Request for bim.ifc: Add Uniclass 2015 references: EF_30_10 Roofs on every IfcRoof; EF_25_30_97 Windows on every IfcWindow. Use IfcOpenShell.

First a look at what the model holds.

```python
import ifcopenshell

model = ifcopenshell.open("bim.ifc")
print(model.schema)
print("classifications:", [c.Name for c in model.by_type("IfcClassification")])
for ifc_class in ("IfcDoor", "IfcRoof", "IfcStair", "IfcWall", "IfcWindow"):
    print(ifc_class, len(model.by_type(ifc_class)))
```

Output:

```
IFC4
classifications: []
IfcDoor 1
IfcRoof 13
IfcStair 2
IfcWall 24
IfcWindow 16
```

```python
import ifcopenshell
import ifcopenshell.api.classification

model = ifcopenshell.open("bim.ifc")

system = ifcopenshell.api.classification.add_classification(model, classification="Uniclass 2015")

codes = {
    "IfcRoof": ("EF_30_10", "Roofs"),
    "IfcWindow": ("EF_25_30_97", "Windows"),
}
for ifc_class, (code, name) in codes.items():
    products = model.by_type(ifc_class)
    ifcopenshell.api.classification.add_reference(
        model, products=products, classification=system, identification=code, name=name
    )
    print(code, len(products))

model.write("bim_updated.ifc")
```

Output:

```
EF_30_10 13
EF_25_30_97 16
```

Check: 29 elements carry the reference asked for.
